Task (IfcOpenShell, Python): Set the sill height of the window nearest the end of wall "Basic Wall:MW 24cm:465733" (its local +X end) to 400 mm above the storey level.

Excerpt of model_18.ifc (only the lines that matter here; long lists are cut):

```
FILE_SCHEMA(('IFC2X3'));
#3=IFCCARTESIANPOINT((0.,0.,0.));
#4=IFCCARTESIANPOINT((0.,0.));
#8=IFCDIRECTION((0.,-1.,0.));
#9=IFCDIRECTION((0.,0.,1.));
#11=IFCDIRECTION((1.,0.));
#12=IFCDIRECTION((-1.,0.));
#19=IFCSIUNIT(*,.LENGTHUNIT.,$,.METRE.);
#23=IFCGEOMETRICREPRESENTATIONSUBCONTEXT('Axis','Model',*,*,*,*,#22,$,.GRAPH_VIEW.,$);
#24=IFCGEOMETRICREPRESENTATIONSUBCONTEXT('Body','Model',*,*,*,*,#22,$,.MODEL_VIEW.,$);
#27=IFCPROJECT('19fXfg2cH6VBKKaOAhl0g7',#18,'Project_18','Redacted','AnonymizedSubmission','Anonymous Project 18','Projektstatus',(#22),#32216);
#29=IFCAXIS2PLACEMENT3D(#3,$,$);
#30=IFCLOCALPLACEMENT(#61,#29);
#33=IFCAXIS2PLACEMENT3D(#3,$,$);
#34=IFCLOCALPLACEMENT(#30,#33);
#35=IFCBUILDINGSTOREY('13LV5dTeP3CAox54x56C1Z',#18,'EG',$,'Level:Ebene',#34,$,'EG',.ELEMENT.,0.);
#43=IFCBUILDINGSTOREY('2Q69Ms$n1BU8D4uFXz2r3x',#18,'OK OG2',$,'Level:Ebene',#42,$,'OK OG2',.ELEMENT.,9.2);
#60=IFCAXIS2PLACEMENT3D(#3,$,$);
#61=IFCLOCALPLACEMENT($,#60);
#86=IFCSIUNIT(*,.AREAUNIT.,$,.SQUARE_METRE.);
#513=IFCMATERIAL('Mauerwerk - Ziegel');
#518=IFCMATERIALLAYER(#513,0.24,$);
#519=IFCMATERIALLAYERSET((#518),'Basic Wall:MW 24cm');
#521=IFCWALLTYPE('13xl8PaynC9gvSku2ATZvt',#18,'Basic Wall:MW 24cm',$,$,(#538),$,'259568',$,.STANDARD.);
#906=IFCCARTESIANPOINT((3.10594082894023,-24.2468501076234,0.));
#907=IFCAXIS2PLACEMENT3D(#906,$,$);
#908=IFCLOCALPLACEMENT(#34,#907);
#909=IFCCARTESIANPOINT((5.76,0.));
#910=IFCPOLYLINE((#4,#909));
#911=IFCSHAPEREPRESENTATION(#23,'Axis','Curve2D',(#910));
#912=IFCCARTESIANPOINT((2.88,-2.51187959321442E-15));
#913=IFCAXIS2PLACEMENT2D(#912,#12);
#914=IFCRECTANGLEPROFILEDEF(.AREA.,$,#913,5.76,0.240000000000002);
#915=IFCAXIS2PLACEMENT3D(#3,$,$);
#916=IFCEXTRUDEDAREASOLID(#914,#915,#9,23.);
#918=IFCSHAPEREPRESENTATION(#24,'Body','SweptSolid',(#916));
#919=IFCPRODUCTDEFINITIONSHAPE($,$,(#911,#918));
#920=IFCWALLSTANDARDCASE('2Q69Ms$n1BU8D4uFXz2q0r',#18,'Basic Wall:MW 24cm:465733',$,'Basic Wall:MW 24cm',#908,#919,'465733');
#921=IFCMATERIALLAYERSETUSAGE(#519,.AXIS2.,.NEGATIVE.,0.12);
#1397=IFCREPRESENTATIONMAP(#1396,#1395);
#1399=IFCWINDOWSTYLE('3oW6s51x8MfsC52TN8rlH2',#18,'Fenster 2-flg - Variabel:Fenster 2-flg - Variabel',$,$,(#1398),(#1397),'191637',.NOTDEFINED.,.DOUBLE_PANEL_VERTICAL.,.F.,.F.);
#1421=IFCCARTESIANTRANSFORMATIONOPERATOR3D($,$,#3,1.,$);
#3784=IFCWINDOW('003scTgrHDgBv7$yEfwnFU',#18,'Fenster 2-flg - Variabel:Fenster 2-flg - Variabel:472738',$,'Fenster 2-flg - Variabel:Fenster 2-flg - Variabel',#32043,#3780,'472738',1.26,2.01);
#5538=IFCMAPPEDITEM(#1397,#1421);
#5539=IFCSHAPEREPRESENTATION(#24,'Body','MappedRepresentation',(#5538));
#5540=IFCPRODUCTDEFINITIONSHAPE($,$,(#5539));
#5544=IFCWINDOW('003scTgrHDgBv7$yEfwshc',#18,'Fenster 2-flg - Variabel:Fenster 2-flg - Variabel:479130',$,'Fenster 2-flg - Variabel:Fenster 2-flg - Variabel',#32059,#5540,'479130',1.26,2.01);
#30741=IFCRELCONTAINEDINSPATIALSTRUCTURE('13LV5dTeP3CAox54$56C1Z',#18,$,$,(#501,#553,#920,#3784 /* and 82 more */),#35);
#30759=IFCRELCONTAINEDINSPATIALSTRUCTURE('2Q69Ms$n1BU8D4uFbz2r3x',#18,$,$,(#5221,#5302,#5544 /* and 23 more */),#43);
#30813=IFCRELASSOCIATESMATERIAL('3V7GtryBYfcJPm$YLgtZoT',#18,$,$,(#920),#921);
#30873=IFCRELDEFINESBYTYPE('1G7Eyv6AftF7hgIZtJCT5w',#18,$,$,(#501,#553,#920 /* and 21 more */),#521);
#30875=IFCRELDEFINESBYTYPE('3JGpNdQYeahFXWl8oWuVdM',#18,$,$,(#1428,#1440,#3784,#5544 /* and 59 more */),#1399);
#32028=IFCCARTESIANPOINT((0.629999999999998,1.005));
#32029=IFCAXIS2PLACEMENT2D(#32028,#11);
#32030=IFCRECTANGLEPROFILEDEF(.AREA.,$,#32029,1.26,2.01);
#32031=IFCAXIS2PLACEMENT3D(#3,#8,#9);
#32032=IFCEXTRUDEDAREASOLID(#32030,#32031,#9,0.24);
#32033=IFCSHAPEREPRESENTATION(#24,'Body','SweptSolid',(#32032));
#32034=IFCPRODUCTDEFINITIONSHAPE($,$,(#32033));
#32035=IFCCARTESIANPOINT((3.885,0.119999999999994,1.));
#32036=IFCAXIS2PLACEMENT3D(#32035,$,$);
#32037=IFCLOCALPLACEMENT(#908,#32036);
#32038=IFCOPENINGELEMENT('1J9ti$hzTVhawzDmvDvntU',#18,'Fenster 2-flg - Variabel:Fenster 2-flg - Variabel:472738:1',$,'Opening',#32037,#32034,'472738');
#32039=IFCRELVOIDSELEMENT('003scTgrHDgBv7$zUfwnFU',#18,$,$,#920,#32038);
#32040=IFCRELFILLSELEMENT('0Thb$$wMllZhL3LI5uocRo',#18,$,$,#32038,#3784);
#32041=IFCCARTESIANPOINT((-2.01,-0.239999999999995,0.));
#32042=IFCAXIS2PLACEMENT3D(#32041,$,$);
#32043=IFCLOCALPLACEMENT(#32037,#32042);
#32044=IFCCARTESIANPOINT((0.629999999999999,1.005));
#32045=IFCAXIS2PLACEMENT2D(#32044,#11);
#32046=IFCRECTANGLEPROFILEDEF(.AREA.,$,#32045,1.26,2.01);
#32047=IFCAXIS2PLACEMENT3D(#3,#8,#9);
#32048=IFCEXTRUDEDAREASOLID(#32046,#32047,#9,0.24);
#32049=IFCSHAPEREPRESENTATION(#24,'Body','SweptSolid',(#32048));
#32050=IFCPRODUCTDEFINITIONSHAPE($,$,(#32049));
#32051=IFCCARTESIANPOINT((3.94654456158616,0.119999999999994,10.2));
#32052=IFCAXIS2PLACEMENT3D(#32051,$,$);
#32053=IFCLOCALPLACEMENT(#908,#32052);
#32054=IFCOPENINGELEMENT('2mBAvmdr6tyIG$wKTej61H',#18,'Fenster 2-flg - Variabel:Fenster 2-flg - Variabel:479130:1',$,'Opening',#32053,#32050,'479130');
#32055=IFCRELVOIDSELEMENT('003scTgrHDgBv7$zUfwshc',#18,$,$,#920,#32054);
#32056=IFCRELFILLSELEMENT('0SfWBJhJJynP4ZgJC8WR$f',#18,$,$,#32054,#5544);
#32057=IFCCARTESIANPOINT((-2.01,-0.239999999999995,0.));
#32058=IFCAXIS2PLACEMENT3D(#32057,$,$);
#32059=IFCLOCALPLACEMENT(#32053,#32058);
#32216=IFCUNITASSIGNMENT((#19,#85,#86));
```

```python
import numpy as np
import ifcopenshell
import ifcopenshell.api.geometry
import ifcopenshell.geom
import ifcopenshell.util.element
import ifcopenshell.util.placement
import ifcopenshell.util.shape
import ifcopenshell.util.unit

model = ifcopenshell.open("model_18.ifc")
unit_scale = ifcopenshell.util.unit.calculate_unit_scale(model)

window = model.by_guid("003scTgrHDgBv7$yEfwshc")
opening = window.FillsVoids[0].RelatingOpeningElement
storey = ifcopenshell.util.element.get_container(window, ifc_class="IfcBuildingStorey")
level = ifcopenshell.util.placement.get_local_placement(storey.ObjectPlacement)[2, 3]

# The opening's origin need not be at the sill, so measure its lowest point.
shape = ifcopenshell.geom.create_shape(ifcopenshell.geom.settings(), opening)
bottom = ifcopenshell.util.shape.get_shape_bottom_elevation(shape, shape.geometry) / unit_scale
dz = level + 0.4 / unit_scale - bottom

shift = np.array([0.0, 0.0, dz])
# The window is placed relative to its opening, so it follows when the opening moves.
matrix = ifcopenshell.util.placement.get_local_placement(opening.ObjectPlacement)
matrix[:3, 3] += shift
ifcopenshell.api.geometry.edit_object_placement(
    model, product=opening, matrix=matrix, is_si=False, should_transform_children=True
)

print(f"moved by {dz * unit_scale:+.3f} m")

model.write("model_18_edited.ifc")
```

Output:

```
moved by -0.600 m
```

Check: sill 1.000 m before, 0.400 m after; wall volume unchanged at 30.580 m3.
